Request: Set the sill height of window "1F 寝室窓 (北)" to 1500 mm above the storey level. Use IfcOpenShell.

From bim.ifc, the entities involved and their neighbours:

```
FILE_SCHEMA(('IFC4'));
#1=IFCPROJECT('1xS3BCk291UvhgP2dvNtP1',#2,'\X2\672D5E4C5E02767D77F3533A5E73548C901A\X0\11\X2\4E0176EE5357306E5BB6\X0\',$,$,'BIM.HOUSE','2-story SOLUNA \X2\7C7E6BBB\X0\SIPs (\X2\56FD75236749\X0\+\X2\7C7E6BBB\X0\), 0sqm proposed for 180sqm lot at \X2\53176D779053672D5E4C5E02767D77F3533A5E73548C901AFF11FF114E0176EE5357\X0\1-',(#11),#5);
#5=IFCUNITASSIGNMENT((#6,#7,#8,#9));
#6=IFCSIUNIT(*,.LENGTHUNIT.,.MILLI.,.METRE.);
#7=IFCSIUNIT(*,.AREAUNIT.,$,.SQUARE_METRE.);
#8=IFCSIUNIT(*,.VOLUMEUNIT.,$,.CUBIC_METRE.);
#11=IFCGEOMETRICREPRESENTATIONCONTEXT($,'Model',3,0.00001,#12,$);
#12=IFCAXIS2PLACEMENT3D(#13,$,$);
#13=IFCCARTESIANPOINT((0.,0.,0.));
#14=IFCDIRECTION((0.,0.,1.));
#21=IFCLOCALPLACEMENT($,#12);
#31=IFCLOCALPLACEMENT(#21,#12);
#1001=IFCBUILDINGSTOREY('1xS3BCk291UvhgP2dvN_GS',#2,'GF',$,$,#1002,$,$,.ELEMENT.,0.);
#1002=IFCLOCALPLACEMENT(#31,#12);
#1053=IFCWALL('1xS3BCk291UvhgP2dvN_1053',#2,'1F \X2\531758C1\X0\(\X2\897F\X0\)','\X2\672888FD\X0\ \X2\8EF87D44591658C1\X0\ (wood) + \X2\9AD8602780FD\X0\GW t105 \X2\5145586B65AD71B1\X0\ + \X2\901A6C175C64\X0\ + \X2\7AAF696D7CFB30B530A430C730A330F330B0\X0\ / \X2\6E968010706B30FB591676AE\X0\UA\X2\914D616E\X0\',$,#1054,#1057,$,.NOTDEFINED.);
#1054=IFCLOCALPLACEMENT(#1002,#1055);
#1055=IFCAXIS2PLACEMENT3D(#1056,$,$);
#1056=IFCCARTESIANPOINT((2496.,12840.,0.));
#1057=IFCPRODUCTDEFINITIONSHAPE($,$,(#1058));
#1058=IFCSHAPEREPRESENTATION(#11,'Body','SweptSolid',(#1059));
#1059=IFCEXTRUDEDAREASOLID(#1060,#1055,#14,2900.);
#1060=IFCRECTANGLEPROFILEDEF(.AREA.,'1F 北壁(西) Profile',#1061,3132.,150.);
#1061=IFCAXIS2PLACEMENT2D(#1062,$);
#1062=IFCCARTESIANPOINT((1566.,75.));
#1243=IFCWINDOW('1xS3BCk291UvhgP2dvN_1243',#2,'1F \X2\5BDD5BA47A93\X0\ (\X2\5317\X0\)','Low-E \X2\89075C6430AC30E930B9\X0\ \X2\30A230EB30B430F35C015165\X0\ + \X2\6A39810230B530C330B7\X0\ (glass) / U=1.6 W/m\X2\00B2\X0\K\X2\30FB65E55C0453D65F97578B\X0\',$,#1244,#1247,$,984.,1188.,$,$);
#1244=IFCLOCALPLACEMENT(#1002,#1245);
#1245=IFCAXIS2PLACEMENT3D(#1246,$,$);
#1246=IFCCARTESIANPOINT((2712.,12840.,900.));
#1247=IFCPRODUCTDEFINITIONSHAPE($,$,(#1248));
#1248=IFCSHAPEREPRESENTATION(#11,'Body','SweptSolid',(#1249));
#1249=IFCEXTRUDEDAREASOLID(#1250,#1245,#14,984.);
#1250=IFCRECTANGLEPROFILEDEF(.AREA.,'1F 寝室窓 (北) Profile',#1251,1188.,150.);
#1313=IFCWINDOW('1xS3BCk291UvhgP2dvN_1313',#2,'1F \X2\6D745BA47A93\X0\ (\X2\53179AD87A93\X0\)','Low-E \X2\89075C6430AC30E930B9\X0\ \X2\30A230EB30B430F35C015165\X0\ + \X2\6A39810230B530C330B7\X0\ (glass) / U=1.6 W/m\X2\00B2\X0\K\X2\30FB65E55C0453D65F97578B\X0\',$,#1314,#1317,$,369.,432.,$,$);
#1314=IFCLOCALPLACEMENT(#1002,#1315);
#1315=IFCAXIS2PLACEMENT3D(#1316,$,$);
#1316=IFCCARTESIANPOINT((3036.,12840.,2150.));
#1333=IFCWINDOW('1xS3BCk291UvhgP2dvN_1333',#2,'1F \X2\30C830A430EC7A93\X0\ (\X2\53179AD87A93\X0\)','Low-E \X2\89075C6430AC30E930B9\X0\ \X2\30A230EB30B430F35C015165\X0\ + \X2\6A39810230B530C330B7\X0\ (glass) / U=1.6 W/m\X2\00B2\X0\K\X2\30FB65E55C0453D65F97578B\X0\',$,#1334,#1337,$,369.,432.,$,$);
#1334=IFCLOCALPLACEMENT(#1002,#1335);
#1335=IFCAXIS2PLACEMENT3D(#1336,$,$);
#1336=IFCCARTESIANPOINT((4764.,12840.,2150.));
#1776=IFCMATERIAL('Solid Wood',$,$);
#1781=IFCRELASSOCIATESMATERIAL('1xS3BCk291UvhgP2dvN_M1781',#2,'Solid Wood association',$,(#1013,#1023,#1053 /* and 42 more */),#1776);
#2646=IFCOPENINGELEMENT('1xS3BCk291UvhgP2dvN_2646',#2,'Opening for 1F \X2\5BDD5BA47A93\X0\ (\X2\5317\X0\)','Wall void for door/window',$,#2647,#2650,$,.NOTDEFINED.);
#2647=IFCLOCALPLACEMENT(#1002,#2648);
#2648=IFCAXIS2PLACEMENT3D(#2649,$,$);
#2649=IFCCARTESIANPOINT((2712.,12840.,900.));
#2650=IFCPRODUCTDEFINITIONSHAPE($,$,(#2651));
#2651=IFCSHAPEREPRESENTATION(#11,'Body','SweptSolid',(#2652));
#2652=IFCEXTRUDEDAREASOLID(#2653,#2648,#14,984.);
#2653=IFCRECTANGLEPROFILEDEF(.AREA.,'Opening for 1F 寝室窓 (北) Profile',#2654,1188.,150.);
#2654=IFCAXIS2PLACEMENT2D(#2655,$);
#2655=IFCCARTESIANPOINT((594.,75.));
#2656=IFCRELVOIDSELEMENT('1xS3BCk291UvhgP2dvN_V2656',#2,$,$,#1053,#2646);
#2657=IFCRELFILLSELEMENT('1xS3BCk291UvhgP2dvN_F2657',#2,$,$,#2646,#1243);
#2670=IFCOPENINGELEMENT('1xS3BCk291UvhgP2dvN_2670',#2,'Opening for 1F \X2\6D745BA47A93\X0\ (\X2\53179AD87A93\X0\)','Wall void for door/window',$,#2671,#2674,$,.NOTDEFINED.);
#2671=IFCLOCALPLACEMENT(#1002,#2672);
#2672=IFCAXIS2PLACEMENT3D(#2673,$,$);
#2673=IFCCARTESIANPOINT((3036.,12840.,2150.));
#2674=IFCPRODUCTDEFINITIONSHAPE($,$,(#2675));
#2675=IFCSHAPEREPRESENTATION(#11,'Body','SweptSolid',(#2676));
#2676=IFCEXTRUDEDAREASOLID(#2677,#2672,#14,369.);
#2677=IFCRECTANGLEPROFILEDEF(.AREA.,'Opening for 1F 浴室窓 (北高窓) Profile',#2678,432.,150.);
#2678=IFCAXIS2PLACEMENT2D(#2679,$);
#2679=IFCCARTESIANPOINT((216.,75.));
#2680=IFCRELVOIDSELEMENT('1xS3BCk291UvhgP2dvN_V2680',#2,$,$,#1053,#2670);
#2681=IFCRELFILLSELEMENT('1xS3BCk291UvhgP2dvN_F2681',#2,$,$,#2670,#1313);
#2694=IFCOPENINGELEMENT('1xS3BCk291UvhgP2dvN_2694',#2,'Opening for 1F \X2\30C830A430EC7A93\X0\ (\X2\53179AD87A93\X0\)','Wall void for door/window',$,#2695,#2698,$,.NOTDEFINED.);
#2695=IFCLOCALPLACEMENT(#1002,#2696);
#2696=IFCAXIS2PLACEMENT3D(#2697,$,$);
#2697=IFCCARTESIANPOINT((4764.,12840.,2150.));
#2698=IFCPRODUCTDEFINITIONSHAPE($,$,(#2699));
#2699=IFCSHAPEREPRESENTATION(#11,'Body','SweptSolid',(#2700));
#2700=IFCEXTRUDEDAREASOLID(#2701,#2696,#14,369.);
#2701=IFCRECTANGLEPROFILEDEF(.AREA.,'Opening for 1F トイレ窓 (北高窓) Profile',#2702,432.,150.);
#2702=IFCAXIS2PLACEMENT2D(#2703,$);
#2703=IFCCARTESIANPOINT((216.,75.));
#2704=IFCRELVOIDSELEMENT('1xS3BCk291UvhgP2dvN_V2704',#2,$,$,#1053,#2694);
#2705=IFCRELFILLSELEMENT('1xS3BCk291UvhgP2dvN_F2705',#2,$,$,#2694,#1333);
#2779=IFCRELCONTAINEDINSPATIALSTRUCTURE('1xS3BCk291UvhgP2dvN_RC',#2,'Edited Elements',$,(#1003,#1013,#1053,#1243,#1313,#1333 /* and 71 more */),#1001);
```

```python
import numpy as np
import ifcopenshell
import ifcopenshell.api.geometry
import ifcopenshell.geom
import ifcopenshell.util.element
import ifcopenshell.util.placement
import ifcopenshell.util.shape
import ifcopenshell.util.unit

model = ifcopenshell.open("bim.ifc")
unit_scale = ifcopenshell.util.unit.calculate_unit_scale(model)

window = model.by_guid("1xS3BCk291UvhgP2dvN_1243")
opening = window.FillsVoids[0].RelatingOpeningElement
storey = ifcopenshell.util.element.get_container(window, ifc_class="IfcBuildingStorey")
level = ifcopenshell.util.placement.get_local_placement(storey.ObjectPlacement)[2, 3]

# The opening's origin need not be at the sill, so measure its lowest point.
shape = ifcopenshell.geom.create_shape(ifcopenshell.geom.settings(), opening)
bottom = ifcopenshell.util.shape.get_shape_bottom_elevation(shape, shape.geometry) / unit_scale
dz = level + 1500.0 - bottom

shift = np.array([0.0, 0.0, dz])
# The window is not placed relative to its opening, so move both.
for product in (opening, window):
    matrix = ifcopenshell.util.placement.get_local_placement(product.ObjectPlacement)
    matrix[:3, 3] += shift
    ifcopenshell.api.geometry.edit_object_placement(model, product=product, matrix=matrix, is_si=False)

print(f"moved by {dz * unit_scale:+.3f} m")

model.write("bim-out.ifc")
```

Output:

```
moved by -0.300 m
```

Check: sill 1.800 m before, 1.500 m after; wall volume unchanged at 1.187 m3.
